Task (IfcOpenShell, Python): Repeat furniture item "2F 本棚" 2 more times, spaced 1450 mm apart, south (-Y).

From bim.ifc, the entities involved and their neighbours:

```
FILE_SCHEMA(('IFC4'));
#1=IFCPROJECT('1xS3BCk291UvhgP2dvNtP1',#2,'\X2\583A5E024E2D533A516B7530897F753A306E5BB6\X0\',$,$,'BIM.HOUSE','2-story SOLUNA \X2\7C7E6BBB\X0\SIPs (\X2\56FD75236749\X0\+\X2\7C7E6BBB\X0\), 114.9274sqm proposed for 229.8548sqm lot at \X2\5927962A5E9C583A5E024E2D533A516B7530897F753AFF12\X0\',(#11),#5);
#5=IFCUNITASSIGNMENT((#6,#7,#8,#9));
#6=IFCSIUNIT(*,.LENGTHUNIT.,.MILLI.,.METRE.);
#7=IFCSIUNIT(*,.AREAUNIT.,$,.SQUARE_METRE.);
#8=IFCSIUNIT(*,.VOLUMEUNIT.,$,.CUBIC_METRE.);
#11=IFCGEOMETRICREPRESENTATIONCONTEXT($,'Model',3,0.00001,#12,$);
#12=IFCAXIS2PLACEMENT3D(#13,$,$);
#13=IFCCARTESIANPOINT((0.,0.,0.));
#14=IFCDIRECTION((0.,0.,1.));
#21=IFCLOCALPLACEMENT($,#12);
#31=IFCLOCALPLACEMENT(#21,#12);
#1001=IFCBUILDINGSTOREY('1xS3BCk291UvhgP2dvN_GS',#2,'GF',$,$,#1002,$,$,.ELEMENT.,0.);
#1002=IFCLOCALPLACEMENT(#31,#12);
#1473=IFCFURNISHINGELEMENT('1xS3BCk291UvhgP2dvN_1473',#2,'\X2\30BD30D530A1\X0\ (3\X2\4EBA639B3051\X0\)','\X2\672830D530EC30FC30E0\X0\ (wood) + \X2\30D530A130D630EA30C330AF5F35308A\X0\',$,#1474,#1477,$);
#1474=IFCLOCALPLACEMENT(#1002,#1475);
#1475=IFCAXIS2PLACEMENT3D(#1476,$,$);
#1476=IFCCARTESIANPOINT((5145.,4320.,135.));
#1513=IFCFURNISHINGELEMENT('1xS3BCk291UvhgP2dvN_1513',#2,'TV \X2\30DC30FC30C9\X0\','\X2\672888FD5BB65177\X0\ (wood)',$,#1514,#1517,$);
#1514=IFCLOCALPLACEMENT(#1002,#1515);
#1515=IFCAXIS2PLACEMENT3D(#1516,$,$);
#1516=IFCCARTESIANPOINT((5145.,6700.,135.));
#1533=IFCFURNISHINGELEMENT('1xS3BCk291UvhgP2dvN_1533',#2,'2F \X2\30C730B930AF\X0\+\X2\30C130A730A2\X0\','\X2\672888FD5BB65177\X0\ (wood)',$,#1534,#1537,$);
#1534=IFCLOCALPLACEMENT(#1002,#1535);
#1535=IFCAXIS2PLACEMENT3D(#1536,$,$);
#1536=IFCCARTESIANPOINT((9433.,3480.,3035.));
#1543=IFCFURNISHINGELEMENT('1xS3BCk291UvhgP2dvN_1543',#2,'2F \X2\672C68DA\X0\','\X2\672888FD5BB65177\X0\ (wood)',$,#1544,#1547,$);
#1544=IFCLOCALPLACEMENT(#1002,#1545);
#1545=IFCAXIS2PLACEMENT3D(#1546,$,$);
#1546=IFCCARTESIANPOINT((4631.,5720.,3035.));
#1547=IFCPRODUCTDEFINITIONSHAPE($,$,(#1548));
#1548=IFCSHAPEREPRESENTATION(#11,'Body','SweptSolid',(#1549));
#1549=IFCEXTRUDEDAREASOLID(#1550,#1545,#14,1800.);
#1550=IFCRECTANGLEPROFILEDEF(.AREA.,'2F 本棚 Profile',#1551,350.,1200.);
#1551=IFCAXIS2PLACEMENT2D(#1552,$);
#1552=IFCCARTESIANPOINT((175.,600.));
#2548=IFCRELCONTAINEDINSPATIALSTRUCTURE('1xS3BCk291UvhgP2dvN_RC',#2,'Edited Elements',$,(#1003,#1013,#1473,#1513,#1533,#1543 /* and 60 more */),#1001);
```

```python
import numpy as np
import ifcopenshell
import ifcopenshell.api.geometry
import ifcopenshell.api.root
import ifcopenshell.util.element
import ifcopenshell.util.placement
import ifcopenshell.util.unit

model = ifcopenshell.open("bim.ifc")
unit_scale = ifcopenshell.util.unit.calculate_unit_scale(model)


def reuse_history(source, copy):
    """copy_class also copies each property set's owner history, people and application; keep the originals."""
    for rel in copy.IsDefinedBy:
        if rel.is_a("IfcRelDefinesByProperties") and (history := rel.RelatingPropertyDefinition.OwnerHistory):
            rel.RelatingPropertyDefinition.OwnerHistory = source.OwnerHistory
            ifcopenshell.util.element.remove_deep2(model, history)


source = model.by_id(1543)
base = ifcopenshell.util.placement.get_local_placement(source.ObjectPlacement)
step = np.array([0.0, -1.0, 0.0]) * 1.45 / unit_scale

for i in range(1, 3):
    copy = ifcopenshell.api.root.copy_class(model, product=source)
    copy.Representation = ifcopenshell.util.element.copy_deep(
        model, source.Representation, exclude=["IfcGeometricRepresentationContext", "IfcRepresentationMap"]
    )
    reuse_history(source, copy)
    matrix = base.copy()
    matrix[:3, 3] += i * step
    print("added at", matrix[:3, 3].round(3) + 0.0)
    ifcopenshell.api.geometry.edit_object_placement(model, product=copy, matrix=matrix, is_si=False)

model.write("bim-out.ifc")
```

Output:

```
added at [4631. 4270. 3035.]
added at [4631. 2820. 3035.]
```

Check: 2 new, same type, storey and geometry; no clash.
